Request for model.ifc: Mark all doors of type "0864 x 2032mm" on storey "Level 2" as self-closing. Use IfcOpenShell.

First a look at what the model holds.

```python
import ifcopenshell
import ifcopenshell.util.element

model = ifcopenshell.open("model.ifc")
print(model.schema)
storey = next(s for s in model.by_type("IfcBuildingStorey") if s.Name == "Level 2")
doors = [e for e in ifcopenshell.util.element.get_decomposition(storey) if e.is_a("IfcDoor")]
seen = {}
for e in doors:
    element_type = ifcopenshell.util.element.get_type(e)
    key = (element_type.Name if element_type != e and element_type else None, ifcopenshell.util.element.get_pset(e, "Pset_DoorCommon", "SelfClosing"))
    seen[key] = seen.get(key, 0) + 1
for (name, value), count in sorted(seen.items(), key=str):
    print(count, "x", name, "|", value)
```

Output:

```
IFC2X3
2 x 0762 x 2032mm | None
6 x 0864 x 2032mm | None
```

```python
import ifcopenshell
import ifcopenshell.api.pset
import ifcopenshell.util.element

model = ifcopenshell.open("model.ifc")

storey = next(s for s in model.by_type("IfcBuildingStorey") if s.Name == "Level 2")
doors = [e for e in ifcopenshell.util.element.get_decomposition(storey) if e.is_a("IfcDoor")]

count = 0
for e in doors:
    element_type = ifcopenshell.util.element.get_type(e)
    if element_type in (None, e) or element_type.Name != "0864 x 2032mm":
        continue
    # add_pset returns the element's existing set when there is one.
    pset = ifcopenshell.api.pset.add_pset(model, product=e, name="Pset_DoorCommon")
    ifcopenshell.api.pset.edit_pset(model, pset=pset, properties={"SelfClosing": True})
    count += 1

print(count, "doors updated")

model.write("model_v2.ifc")
```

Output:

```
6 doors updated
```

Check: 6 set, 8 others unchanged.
